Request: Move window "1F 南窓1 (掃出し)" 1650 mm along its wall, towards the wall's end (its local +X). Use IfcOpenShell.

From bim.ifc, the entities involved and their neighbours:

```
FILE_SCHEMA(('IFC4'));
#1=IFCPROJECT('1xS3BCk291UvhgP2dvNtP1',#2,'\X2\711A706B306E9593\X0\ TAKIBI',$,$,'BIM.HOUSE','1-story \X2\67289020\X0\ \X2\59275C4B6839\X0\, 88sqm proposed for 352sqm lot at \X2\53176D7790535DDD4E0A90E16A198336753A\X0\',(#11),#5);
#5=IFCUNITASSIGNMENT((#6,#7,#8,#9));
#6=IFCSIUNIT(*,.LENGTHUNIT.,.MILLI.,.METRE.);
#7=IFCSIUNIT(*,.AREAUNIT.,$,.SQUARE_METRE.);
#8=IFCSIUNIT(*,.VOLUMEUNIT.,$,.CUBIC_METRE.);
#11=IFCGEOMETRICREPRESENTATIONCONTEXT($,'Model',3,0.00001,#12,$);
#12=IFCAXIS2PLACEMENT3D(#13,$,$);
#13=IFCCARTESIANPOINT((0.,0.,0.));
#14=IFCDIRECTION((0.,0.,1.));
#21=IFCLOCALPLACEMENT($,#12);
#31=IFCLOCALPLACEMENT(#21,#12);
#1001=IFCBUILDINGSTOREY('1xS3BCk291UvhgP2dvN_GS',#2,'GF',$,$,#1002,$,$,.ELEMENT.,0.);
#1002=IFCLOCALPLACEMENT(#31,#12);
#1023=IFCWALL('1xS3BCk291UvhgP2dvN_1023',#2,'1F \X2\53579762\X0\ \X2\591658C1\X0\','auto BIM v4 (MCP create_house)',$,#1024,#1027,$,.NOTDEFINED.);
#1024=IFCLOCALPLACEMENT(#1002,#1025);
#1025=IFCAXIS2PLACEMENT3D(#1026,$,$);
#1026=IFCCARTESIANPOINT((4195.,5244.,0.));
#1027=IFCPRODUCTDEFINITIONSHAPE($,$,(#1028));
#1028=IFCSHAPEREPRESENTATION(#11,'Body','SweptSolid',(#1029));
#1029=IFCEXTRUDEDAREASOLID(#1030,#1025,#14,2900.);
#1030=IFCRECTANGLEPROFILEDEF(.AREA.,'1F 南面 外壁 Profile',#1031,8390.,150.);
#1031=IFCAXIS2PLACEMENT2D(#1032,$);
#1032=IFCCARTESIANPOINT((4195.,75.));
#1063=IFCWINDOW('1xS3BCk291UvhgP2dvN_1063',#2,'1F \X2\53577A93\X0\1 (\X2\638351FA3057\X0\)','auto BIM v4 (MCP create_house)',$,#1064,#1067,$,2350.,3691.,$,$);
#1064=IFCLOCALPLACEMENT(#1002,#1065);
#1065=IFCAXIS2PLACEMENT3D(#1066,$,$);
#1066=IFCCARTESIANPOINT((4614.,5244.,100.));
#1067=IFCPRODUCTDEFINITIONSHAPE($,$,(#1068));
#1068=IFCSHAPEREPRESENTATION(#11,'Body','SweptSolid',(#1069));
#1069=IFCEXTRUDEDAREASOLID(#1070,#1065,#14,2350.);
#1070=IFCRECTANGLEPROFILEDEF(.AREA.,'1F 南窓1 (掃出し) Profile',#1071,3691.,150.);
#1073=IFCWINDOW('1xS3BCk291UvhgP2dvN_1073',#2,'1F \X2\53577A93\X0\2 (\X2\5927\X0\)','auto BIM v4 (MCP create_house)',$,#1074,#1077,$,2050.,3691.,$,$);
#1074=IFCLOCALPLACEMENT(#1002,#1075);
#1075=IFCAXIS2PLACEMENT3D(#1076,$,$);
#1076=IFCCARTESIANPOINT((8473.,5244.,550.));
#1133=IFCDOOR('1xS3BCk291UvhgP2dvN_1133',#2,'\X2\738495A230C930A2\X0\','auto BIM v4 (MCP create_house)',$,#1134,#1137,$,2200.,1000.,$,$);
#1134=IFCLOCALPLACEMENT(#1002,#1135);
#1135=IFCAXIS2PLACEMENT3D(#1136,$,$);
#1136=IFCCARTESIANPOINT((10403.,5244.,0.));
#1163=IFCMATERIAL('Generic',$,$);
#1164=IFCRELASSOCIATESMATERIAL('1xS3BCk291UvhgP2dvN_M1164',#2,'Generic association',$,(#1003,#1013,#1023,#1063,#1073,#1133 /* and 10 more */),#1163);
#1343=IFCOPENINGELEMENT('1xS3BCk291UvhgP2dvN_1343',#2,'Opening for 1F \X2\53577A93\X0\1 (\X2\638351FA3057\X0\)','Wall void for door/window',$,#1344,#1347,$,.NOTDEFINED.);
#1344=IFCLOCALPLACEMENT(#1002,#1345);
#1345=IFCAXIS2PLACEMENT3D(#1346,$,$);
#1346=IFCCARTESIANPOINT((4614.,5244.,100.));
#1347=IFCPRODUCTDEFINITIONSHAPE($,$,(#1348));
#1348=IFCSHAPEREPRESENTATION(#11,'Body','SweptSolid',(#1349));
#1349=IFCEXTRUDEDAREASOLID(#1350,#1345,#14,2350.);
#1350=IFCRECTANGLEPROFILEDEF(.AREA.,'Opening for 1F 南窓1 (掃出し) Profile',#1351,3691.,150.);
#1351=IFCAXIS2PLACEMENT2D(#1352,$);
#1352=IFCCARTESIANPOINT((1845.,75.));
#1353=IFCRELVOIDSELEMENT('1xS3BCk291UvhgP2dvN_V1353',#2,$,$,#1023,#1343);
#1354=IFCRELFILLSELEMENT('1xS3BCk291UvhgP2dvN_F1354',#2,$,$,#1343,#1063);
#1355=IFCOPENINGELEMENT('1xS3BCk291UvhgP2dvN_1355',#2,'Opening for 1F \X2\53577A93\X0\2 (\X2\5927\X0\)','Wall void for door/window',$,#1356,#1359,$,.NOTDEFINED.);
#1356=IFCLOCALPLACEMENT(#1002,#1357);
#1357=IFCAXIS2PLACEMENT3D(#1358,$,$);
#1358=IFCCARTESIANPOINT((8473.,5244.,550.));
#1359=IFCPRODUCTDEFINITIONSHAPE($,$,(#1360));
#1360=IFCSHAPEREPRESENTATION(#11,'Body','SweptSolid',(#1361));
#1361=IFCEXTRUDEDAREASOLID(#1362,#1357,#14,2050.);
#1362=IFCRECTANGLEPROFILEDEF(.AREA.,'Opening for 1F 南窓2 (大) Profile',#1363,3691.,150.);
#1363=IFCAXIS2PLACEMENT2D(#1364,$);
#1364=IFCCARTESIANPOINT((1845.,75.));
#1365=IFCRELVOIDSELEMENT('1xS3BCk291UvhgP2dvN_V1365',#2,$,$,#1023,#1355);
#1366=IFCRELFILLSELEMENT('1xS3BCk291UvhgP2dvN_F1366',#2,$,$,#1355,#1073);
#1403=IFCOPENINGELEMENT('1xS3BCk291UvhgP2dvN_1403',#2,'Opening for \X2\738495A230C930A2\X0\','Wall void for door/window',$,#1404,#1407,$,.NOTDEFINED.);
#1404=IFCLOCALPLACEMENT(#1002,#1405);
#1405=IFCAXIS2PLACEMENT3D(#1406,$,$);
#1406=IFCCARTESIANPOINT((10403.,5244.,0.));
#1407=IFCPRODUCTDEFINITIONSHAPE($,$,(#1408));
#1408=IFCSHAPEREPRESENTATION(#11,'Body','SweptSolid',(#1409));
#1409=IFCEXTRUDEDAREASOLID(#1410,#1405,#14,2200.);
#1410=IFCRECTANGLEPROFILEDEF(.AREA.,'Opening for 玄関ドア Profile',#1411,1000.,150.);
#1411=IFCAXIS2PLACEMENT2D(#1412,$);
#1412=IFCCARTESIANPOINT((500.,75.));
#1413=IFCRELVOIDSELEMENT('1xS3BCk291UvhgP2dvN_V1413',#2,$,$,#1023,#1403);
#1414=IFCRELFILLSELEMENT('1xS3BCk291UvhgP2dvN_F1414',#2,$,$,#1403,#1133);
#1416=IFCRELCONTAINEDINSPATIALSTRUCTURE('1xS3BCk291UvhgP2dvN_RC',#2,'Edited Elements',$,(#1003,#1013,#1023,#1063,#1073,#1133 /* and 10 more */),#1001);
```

```python
import ifcopenshell
import ifcopenshell.api.geometry
import ifcopenshell.util.placement

model = ifcopenshell.open("bim.ifc")

window = model.by_guid("1xS3BCk291UvhgP2dvN_1063")
opening = window.FillsVoids[0].RelatingOpeningElement
wall = opening.VoidsElements[0].RelatingBuildingElement

wall_matrix = ifcopenshell.util.placement.get_local_placement(wall.ObjectPlacement)
shift = wall_matrix[:3, 0] * 1650.0
before = ifcopenshell.util.placement.get_local_placement(window.ObjectPlacement)[:3, 3].copy()

# The window is not placed relative to its opening, so move both.
for product in (opening, window):
    matrix = ifcopenshell.util.placement.get_local_placement(product.ObjectPlacement)
    matrix[:3, 3] += shift
    ifcopenshell.api.geometry.edit_object_placement(model, product=product, matrix=matrix, is_si=False)

after = ifcopenshell.util.placement.get_local_placement(window.ObjectPlacement)[:3, 3]
print("window moved by", (after - before).round(3) + 0.0)

model.write("bim_updated.ifc")
```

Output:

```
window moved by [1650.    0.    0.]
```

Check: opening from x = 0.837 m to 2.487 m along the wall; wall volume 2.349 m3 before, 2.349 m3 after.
